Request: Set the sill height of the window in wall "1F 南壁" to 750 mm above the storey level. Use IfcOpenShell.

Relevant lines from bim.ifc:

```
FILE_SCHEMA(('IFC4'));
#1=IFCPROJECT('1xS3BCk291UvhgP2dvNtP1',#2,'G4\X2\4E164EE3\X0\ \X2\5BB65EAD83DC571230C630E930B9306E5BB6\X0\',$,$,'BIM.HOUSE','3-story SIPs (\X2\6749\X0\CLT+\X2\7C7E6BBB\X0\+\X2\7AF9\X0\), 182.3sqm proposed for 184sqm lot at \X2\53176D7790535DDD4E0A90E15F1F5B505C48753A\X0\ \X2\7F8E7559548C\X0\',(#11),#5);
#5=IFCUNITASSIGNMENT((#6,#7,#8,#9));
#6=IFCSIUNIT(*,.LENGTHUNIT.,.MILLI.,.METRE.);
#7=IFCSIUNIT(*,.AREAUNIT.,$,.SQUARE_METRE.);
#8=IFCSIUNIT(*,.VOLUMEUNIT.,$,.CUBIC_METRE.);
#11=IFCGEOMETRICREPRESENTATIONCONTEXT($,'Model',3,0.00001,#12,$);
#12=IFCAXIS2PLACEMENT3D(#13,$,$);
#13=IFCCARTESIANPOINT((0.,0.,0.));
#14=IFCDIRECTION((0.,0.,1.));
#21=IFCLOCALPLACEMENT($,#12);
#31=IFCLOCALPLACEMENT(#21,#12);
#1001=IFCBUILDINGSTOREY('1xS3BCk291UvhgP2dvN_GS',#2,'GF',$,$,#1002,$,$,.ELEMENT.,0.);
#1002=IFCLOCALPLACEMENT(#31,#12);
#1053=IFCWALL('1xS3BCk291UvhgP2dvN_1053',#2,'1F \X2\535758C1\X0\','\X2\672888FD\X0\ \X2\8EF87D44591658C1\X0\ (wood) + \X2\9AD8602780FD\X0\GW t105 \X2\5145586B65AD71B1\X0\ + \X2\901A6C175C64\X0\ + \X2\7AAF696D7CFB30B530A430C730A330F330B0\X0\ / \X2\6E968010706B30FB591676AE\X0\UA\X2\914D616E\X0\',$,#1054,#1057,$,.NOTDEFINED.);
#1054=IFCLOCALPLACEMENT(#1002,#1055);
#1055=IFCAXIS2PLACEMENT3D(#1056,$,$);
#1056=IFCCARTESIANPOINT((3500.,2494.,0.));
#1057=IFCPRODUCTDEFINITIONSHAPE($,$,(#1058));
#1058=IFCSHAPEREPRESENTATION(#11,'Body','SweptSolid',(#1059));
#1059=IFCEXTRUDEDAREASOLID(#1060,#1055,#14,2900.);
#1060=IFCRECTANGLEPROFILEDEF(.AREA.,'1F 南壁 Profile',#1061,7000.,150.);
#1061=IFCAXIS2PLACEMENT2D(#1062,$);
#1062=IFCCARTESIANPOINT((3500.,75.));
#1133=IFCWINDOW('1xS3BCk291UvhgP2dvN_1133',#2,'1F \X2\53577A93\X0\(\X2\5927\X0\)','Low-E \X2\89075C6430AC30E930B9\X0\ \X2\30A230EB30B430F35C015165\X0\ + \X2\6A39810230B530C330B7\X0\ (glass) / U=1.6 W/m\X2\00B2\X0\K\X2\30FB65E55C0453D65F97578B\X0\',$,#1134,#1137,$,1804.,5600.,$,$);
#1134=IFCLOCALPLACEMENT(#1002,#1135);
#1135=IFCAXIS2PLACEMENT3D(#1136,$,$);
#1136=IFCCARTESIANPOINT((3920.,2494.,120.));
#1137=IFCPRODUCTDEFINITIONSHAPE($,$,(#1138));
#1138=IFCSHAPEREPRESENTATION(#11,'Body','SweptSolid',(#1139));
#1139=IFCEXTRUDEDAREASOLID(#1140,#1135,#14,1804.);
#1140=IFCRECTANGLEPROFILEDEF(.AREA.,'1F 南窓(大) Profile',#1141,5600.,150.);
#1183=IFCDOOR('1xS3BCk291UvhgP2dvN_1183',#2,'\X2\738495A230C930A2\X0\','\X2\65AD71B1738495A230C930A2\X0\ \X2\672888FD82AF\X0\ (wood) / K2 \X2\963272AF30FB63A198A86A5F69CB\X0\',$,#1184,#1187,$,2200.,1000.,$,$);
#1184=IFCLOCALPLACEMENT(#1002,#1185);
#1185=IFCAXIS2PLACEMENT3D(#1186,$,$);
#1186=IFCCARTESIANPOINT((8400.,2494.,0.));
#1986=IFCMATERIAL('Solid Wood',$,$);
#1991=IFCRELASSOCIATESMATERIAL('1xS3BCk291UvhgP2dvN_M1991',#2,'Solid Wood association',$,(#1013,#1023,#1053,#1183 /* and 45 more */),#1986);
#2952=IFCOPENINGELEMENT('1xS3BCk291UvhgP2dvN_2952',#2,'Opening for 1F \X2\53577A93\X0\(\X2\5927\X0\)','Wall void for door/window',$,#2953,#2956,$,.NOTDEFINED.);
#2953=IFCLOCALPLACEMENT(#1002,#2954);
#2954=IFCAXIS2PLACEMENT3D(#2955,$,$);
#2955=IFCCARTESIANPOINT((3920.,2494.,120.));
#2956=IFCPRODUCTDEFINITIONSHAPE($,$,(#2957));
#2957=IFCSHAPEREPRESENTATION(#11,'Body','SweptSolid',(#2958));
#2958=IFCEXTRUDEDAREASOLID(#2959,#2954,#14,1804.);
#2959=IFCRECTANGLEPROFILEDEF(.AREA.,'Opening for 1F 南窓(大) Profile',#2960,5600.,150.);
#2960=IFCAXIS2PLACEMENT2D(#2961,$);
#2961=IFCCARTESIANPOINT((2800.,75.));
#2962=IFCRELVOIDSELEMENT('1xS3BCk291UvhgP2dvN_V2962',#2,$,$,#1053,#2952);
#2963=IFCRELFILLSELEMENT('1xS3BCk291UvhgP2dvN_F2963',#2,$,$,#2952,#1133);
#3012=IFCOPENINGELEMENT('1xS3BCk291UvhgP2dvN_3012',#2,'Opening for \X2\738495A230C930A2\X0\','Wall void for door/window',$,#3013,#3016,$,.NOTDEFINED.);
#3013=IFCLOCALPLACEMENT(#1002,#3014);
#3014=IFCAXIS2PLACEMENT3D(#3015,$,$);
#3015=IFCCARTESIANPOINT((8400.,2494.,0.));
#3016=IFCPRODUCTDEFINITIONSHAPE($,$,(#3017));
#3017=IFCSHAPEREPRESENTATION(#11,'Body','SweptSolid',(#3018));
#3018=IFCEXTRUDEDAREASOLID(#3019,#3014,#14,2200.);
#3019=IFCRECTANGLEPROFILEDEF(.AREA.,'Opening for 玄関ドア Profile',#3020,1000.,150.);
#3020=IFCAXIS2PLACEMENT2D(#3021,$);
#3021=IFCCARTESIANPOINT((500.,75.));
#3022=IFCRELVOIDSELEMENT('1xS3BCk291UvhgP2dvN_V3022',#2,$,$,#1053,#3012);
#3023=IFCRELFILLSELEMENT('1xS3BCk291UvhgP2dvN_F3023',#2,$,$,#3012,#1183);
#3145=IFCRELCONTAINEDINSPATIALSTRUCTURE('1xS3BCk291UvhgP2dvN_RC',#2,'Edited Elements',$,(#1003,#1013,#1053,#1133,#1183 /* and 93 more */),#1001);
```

```python
import numpy as np
import ifcopenshell
import ifcopenshell.api.geometry
import ifcopenshell.geom
import ifcopenshell.util.element
import ifcopenshell.util.placement
import ifcopenshell.util.shape
import ifcopenshell.util.unit

model = ifcopenshell.open("bim.ifc")
unit_scale = ifcopenshell.util.unit.calculate_unit_scale(model)

window = model.by_guid("1xS3BCk291UvhgP2dvN_1133")
opening = window.FillsVoids[0].RelatingOpeningElement
storey = ifcopenshell.util.element.get_container(window, ifc_class="IfcBuildingStorey")
level = ifcopenshell.util.placement.get_local_placement(storey.ObjectPlacement)[2, 3]

# The opening's origin need not be at the sill, so measure its lowest point.
shape = ifcopenshell.geom.create_shape(ifcopenshell.geom.settings(), opening)
bottom = ifcopenshell.util.shape.get_shape_bottom_elevation(shape, shape.geometry) / unit_scale
dz = level + 750.0 - bottom

shift = np.array([0.0, 0.0, dz])
# The window is not placed relative to its opening, so move both.
for product in (opening, window):
    matrix = ifcopenshell.util.placement.get_local_placement(product.ObjectPlacement)
    matrix[:3, 3] += shift
    ifcopenshell.api.geometry.edit_object_placement(model, product=product, matrix=matrix, is_si=False)

print(f"moved by {dz * unit_scale:+.3f} m")

model.write("bim_rev.ifc")
```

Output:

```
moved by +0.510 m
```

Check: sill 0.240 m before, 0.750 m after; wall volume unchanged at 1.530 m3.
